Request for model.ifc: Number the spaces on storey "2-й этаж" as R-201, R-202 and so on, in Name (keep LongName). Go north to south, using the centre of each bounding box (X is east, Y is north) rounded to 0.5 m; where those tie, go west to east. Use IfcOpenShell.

First a look at what the model holds.

```python
import ifcopenshell
import ifcopenshell.util.element
import ifcopenshell.util.placement

model = ifcopenshell.open("model.ifc")
print(model.schema)
storey = next(s for s in model.by_type("IfcBuildingStorey") if s.Name == "2-й этаж")
spaces = [e for e in ifcopenshell.util.element.get_decomposition(storey) if e.is_a("IfcSpace")]
for e in sorted(spaces, key=lambda e: e.id()):
    origin = ifcopenshell.util.placement.get_local_placement(e.ObjectPlacement)[:3, 3]
    print(e.id(), e.Name, e.LongName, origin.round(2) + 0.0, sep=" | ")
```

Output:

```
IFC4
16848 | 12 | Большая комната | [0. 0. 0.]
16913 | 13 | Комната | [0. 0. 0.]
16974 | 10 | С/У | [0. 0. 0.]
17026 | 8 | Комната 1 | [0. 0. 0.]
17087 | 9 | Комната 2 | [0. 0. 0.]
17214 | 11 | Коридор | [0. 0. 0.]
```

```python
import ifcopenshell
import ifcopenshell.geom
import ifcopenshell.util.element
import ifcopenshell.util.shape

model = ifcopenshell.open("model.ifc")
settings = ifcopenshell.geom.settings()
settings.set("use-world-coords", True)


def centre(element):
    shape = ifcopenshell.geom.create_shape(settings, element)
    return ifcopenshell.util.shape.get_bbox_centroid(shape.geometry)


storey = next(s for s in model.by_type("IfcBuildingStorey") if s.Name == "2-й этаж")
spaces = [e for e in ifcopenshell.util.element.get_decomposition(storey) if e.is_a("IfcSpace")]

# Insertion points can sit at a corner or the storey origin, so sort by the geometry (in metres).
centres = {e: centre(e) for e in spaces}
spaces.sort(key=lambda e: (-round(centres[e][1] / 0.5), centres[e][0]))

for i, e in enumerate(spaces, start=1):
    number = f"R-2{i:02d}"
    e.Name = number
    print(e.id(), number)

model.write("model-out.ifc")
```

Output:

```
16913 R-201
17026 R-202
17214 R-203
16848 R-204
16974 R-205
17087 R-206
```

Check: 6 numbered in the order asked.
